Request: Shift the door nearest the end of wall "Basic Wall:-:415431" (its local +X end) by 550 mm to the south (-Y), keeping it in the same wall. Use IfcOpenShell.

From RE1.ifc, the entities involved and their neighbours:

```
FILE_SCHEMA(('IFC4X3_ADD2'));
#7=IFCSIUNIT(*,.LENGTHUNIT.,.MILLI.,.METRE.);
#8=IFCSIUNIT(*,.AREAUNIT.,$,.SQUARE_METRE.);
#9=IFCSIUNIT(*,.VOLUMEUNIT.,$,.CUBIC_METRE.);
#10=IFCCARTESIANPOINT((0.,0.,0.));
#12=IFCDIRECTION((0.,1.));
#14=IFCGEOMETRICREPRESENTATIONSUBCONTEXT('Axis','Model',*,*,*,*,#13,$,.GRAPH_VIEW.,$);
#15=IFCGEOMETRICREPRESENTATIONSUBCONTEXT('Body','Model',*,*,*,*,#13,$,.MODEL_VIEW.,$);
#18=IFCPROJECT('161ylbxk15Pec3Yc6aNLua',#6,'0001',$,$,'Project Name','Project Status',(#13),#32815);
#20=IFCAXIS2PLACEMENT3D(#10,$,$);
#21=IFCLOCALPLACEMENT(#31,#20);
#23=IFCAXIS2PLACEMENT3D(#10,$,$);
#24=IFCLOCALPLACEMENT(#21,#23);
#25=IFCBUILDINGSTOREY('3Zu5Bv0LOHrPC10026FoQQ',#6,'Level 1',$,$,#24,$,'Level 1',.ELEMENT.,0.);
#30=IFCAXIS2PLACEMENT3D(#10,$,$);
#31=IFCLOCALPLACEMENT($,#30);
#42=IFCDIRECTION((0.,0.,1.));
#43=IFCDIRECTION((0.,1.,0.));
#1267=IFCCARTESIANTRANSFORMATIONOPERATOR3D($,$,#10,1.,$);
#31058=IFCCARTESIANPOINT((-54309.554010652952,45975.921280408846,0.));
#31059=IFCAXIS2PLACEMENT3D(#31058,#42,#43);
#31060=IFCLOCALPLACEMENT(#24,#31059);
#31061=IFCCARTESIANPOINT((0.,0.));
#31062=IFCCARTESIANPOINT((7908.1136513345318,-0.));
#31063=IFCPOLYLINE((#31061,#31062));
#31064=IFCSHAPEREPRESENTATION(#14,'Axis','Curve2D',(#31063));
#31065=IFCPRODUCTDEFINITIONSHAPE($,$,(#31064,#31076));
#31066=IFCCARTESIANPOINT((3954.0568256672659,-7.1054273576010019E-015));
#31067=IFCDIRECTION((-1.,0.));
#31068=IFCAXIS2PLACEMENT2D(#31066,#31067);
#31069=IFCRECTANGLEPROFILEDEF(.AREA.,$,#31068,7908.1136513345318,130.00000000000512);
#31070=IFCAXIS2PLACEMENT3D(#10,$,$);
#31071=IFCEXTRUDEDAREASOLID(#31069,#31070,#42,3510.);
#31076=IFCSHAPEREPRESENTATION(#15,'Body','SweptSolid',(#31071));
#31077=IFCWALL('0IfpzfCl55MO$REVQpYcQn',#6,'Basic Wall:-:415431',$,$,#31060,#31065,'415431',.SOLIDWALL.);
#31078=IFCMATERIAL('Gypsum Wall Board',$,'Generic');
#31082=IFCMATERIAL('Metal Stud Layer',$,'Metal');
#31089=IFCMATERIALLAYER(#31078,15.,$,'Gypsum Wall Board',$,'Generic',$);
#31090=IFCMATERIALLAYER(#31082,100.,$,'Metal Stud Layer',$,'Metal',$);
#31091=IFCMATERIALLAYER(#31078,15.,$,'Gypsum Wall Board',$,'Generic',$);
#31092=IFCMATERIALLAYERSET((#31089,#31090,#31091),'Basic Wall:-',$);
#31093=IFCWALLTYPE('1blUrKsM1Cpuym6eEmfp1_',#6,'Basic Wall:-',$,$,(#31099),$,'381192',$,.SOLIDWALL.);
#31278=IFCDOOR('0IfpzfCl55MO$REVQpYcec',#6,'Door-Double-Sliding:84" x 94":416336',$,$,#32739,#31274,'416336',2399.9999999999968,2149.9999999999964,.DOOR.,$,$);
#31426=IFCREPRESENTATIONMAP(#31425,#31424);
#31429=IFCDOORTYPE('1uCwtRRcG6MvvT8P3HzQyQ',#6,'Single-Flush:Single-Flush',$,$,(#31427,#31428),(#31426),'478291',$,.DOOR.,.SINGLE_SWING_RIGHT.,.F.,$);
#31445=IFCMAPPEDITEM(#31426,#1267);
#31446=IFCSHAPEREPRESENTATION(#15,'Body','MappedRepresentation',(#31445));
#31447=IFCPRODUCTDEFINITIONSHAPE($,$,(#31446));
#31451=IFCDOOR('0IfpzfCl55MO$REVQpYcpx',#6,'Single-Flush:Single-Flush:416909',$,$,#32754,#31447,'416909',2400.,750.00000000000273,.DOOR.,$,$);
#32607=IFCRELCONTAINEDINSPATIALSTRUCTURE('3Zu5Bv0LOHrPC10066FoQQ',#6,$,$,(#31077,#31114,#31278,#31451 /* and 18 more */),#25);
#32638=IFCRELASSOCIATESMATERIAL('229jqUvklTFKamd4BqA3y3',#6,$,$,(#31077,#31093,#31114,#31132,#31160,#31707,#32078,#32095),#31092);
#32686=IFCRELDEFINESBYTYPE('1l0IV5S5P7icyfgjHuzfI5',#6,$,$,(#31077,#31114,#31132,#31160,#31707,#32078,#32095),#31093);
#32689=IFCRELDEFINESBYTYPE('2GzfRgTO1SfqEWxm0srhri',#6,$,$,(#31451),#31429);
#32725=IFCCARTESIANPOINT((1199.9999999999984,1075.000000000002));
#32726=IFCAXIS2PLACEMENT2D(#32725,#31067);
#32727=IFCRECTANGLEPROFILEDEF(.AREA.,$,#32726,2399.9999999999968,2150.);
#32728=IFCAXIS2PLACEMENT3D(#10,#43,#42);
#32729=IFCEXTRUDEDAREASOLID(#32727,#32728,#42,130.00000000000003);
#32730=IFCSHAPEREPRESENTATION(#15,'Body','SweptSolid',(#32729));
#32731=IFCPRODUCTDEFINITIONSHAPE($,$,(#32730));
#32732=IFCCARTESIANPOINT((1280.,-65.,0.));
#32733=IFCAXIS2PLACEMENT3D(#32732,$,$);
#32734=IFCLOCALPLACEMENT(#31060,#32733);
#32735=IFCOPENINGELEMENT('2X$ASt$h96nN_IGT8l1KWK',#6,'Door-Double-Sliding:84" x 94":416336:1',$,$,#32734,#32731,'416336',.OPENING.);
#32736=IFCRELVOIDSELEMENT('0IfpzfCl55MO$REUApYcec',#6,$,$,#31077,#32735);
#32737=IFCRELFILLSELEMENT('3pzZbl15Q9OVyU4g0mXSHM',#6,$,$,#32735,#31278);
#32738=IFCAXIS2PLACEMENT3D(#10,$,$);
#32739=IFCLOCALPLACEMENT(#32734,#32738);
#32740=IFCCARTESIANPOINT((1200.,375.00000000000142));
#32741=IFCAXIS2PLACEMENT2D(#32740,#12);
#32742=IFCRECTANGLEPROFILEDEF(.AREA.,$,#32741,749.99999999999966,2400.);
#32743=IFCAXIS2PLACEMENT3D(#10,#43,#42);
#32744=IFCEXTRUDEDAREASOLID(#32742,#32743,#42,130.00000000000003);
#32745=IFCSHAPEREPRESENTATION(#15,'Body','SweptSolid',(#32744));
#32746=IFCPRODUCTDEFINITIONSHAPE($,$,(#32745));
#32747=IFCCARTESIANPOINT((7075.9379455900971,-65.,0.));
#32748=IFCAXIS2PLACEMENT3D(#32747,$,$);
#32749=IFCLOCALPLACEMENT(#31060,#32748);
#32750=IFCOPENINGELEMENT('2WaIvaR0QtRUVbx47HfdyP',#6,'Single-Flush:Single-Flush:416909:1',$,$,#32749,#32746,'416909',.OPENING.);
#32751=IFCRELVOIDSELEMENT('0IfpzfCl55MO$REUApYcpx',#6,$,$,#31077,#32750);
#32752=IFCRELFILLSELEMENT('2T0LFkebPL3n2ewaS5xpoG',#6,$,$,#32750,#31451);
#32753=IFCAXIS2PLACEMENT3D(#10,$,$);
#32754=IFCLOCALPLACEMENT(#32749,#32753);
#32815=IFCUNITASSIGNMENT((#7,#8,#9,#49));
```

```python
import ifcopenshell
import ifcopenshell.api.geometry
import ifcopenshell.util.placement
import ifcopenshell.util.unit

model = ifcopenshell.open("RE1.ifc")
unit_scale = ifcopenshell.util.unit.calculate_unit_scale(model)

door = model.by_id(31451)
opening = door.FillsVoids[0].RelatingOpeningElement
wall = opening.VoidsElements[0].RelatingBuildingElement

wall_matrix = ifcopenshell.util.placement.get_local_placement(wall.ObjectPlacement)
shift = wall_matrix[:3, 0] * -0.55 / unit_scale
before = ifcopenshell.util.placement.get_local_placement(door.ObjectPlacement)[:3, 3].copy()

# The door is placed relative to its opening, so it follows when the opening moves.
matrix = ifcopenshell.util.placement.get_local_placement(opening.ObjectPlacement)
matrix[:3, 3] += shift
ifcopenshell.api.geometry.edit_object_placement(
    model, product=opening, matrix=matrix, is_si=False, should_transform_children=True
)

after = ifcopenshell.util.placement.get_local_placement(door.ObjectPlacement)[:3, 3]
print("door moved by", (after - before).round(3) + 0.0)

model.write("RE1-out.ifc")
```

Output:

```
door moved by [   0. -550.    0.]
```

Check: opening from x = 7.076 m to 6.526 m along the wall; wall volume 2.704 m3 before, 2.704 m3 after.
